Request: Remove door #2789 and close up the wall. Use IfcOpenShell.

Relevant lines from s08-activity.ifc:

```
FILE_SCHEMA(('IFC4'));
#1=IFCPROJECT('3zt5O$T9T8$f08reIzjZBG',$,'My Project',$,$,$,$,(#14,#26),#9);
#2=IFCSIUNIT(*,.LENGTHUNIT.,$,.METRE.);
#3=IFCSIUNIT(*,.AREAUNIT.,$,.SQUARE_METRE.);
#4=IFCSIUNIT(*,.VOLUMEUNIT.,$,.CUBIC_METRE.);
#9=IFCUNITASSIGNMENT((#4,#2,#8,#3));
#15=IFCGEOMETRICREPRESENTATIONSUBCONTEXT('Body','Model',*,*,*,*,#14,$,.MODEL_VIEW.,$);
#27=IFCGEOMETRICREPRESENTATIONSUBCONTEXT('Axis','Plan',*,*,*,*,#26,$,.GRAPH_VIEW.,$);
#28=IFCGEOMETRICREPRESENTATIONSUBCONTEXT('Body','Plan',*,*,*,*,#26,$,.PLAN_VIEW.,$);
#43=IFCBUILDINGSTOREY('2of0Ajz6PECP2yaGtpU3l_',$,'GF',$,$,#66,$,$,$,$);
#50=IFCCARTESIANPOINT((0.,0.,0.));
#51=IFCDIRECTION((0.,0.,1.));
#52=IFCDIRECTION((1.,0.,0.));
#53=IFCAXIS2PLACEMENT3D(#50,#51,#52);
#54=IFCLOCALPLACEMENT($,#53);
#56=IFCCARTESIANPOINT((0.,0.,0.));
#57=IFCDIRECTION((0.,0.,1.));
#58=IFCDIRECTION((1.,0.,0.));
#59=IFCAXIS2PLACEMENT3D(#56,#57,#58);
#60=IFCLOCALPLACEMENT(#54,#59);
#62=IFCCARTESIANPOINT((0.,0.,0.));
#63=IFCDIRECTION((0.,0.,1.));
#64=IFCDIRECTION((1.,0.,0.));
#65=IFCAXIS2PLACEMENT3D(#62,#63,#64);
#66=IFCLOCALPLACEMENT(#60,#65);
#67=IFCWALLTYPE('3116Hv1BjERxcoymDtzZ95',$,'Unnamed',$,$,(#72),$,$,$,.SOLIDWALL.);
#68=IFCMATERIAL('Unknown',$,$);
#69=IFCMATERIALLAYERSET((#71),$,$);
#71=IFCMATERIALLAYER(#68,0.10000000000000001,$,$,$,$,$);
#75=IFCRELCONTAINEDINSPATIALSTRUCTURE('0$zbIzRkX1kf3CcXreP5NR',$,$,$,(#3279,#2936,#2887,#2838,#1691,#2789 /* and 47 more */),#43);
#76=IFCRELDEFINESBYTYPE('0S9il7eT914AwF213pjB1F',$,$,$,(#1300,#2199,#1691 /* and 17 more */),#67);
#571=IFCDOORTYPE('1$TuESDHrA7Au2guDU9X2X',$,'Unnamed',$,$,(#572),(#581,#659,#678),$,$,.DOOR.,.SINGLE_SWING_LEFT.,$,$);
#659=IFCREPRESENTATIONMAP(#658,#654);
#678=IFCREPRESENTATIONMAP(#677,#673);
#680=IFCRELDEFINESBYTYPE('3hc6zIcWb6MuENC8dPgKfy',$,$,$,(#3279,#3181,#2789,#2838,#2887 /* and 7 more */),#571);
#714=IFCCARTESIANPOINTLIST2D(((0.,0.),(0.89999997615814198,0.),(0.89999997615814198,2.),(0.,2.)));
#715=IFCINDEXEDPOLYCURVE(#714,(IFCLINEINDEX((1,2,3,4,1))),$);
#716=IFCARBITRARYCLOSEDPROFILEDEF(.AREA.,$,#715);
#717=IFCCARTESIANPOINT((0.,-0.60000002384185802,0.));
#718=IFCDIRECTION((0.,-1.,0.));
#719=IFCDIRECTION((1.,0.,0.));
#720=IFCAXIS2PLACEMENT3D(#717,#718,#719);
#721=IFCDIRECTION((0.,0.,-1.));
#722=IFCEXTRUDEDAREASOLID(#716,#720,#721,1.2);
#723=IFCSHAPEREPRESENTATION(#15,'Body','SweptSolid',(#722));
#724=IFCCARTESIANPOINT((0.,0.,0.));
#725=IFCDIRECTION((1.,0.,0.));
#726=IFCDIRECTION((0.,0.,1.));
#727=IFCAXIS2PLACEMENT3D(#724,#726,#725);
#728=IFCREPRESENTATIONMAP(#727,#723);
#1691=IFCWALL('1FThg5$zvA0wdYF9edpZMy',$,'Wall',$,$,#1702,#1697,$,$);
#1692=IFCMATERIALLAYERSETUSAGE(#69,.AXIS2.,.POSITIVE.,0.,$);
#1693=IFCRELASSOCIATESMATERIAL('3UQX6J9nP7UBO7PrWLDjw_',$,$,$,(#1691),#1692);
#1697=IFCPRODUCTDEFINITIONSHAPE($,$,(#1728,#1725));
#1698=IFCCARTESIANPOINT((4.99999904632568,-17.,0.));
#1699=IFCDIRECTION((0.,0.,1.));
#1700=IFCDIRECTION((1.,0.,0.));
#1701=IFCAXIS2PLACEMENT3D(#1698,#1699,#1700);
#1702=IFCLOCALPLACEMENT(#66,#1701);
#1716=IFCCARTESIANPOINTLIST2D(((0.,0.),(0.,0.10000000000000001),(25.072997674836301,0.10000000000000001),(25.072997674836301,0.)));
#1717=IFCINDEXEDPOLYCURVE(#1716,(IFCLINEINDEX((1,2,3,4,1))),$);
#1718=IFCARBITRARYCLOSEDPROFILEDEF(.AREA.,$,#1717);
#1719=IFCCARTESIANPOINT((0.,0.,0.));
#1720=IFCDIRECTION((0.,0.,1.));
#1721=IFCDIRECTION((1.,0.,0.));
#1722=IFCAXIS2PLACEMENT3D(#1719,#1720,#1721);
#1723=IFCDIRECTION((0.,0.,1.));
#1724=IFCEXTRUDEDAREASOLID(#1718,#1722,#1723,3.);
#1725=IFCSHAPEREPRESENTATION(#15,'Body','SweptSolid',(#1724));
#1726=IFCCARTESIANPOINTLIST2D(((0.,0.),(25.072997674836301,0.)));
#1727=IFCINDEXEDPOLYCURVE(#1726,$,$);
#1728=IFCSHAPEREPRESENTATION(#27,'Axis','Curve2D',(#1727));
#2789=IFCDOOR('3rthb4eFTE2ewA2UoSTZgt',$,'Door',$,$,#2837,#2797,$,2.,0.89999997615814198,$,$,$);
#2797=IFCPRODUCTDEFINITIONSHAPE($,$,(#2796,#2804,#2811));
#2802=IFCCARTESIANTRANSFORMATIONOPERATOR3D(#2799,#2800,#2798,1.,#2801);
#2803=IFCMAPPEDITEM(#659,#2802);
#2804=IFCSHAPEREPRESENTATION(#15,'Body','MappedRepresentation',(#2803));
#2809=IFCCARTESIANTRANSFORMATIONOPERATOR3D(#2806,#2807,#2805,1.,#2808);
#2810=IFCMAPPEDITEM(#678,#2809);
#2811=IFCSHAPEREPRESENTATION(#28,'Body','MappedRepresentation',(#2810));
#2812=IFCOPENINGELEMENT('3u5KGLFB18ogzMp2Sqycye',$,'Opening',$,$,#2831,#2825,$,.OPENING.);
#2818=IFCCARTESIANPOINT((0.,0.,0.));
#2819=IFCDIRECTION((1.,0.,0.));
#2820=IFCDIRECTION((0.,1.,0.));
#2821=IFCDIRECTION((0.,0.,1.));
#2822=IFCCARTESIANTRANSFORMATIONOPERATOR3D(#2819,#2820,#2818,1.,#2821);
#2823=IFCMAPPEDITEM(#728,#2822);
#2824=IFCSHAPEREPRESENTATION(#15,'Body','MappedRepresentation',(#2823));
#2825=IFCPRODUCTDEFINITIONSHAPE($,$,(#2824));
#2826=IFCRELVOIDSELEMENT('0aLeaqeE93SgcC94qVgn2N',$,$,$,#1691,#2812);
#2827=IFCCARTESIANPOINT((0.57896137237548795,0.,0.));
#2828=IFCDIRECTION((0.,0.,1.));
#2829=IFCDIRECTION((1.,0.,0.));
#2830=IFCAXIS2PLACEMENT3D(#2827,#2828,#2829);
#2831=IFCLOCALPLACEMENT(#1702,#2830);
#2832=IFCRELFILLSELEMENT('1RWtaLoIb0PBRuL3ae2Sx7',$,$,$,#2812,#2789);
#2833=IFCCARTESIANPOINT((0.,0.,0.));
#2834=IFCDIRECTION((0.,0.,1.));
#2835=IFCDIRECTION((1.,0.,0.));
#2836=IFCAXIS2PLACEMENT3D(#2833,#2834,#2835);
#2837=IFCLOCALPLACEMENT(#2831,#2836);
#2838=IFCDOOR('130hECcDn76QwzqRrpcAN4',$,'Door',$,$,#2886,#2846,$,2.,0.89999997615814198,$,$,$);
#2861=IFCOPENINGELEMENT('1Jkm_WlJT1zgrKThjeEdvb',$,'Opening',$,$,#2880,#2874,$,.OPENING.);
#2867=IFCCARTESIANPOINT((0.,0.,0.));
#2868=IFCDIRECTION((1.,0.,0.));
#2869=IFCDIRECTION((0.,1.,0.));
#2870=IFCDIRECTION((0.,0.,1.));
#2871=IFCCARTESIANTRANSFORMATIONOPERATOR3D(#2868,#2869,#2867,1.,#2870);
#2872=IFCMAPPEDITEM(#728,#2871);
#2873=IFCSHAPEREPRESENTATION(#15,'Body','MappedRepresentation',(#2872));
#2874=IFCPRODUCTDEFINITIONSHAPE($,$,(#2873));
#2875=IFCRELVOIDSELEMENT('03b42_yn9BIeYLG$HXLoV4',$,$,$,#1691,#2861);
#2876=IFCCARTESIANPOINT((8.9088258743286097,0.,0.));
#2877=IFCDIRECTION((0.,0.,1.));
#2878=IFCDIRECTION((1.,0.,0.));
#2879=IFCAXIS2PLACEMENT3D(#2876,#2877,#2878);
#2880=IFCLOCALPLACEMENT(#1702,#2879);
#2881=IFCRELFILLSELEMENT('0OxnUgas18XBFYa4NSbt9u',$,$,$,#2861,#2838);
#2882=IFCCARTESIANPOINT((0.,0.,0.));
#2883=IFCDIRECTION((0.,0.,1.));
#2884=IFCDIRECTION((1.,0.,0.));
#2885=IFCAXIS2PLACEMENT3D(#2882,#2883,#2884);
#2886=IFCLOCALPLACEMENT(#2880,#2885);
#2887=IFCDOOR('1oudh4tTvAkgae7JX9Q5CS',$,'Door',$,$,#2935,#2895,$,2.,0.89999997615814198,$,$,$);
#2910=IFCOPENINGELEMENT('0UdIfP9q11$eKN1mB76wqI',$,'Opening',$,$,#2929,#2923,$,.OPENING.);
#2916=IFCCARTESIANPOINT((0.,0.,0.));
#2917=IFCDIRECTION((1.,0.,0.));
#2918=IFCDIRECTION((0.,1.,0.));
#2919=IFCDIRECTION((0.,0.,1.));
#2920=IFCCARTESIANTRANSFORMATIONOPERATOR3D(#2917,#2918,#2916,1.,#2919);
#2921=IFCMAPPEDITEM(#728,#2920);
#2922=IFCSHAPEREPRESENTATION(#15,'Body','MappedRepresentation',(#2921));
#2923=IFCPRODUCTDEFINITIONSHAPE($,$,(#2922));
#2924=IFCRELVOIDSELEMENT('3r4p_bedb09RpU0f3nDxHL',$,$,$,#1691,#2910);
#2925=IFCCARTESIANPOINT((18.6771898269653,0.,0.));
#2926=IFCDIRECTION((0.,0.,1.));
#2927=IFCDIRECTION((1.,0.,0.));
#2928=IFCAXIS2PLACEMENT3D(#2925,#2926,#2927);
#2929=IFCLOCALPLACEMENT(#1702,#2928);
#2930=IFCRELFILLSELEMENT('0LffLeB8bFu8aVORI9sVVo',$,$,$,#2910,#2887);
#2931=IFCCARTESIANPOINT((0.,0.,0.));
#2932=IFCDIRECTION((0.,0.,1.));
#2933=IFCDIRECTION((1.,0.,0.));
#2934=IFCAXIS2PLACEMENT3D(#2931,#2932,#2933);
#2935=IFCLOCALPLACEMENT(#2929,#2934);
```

```python
import ifcopenshell
import ifcopenshell.api.feature
import ifcopenshell.api.root
import ifcopenshell.geom
import ifcopenshell.util.shape

model = ifcopenshell.open("s08-activity.ifc")
settings = ifcopenshell.geom.settings()


def volume(element):
    """Net volume in cubic metres, openings subtracted."""
    shape = ifcopenshell.geom.create_shape(settings, element)
    return ifcopenshell.util.shape.get_volume(shape.geometry)


door = model.by_id(2789)
opening = door.FillsVoids[0].RelatingOpeningElement
wall = opening.VoidsElements[0].RelatingBuildingElement
before = volume(wall)

ifcopenshell.api.root.remove_product(model, product=door)
ifcopenshell.api.feature.remove_feature(model, feature=opening)

after = volume(wall)

print(f"wall volume {before:.3f} -> {after:.3f} m3")

model.write("s08-activity_edited.ifc")
```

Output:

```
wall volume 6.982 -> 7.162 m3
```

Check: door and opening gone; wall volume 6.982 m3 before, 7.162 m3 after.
